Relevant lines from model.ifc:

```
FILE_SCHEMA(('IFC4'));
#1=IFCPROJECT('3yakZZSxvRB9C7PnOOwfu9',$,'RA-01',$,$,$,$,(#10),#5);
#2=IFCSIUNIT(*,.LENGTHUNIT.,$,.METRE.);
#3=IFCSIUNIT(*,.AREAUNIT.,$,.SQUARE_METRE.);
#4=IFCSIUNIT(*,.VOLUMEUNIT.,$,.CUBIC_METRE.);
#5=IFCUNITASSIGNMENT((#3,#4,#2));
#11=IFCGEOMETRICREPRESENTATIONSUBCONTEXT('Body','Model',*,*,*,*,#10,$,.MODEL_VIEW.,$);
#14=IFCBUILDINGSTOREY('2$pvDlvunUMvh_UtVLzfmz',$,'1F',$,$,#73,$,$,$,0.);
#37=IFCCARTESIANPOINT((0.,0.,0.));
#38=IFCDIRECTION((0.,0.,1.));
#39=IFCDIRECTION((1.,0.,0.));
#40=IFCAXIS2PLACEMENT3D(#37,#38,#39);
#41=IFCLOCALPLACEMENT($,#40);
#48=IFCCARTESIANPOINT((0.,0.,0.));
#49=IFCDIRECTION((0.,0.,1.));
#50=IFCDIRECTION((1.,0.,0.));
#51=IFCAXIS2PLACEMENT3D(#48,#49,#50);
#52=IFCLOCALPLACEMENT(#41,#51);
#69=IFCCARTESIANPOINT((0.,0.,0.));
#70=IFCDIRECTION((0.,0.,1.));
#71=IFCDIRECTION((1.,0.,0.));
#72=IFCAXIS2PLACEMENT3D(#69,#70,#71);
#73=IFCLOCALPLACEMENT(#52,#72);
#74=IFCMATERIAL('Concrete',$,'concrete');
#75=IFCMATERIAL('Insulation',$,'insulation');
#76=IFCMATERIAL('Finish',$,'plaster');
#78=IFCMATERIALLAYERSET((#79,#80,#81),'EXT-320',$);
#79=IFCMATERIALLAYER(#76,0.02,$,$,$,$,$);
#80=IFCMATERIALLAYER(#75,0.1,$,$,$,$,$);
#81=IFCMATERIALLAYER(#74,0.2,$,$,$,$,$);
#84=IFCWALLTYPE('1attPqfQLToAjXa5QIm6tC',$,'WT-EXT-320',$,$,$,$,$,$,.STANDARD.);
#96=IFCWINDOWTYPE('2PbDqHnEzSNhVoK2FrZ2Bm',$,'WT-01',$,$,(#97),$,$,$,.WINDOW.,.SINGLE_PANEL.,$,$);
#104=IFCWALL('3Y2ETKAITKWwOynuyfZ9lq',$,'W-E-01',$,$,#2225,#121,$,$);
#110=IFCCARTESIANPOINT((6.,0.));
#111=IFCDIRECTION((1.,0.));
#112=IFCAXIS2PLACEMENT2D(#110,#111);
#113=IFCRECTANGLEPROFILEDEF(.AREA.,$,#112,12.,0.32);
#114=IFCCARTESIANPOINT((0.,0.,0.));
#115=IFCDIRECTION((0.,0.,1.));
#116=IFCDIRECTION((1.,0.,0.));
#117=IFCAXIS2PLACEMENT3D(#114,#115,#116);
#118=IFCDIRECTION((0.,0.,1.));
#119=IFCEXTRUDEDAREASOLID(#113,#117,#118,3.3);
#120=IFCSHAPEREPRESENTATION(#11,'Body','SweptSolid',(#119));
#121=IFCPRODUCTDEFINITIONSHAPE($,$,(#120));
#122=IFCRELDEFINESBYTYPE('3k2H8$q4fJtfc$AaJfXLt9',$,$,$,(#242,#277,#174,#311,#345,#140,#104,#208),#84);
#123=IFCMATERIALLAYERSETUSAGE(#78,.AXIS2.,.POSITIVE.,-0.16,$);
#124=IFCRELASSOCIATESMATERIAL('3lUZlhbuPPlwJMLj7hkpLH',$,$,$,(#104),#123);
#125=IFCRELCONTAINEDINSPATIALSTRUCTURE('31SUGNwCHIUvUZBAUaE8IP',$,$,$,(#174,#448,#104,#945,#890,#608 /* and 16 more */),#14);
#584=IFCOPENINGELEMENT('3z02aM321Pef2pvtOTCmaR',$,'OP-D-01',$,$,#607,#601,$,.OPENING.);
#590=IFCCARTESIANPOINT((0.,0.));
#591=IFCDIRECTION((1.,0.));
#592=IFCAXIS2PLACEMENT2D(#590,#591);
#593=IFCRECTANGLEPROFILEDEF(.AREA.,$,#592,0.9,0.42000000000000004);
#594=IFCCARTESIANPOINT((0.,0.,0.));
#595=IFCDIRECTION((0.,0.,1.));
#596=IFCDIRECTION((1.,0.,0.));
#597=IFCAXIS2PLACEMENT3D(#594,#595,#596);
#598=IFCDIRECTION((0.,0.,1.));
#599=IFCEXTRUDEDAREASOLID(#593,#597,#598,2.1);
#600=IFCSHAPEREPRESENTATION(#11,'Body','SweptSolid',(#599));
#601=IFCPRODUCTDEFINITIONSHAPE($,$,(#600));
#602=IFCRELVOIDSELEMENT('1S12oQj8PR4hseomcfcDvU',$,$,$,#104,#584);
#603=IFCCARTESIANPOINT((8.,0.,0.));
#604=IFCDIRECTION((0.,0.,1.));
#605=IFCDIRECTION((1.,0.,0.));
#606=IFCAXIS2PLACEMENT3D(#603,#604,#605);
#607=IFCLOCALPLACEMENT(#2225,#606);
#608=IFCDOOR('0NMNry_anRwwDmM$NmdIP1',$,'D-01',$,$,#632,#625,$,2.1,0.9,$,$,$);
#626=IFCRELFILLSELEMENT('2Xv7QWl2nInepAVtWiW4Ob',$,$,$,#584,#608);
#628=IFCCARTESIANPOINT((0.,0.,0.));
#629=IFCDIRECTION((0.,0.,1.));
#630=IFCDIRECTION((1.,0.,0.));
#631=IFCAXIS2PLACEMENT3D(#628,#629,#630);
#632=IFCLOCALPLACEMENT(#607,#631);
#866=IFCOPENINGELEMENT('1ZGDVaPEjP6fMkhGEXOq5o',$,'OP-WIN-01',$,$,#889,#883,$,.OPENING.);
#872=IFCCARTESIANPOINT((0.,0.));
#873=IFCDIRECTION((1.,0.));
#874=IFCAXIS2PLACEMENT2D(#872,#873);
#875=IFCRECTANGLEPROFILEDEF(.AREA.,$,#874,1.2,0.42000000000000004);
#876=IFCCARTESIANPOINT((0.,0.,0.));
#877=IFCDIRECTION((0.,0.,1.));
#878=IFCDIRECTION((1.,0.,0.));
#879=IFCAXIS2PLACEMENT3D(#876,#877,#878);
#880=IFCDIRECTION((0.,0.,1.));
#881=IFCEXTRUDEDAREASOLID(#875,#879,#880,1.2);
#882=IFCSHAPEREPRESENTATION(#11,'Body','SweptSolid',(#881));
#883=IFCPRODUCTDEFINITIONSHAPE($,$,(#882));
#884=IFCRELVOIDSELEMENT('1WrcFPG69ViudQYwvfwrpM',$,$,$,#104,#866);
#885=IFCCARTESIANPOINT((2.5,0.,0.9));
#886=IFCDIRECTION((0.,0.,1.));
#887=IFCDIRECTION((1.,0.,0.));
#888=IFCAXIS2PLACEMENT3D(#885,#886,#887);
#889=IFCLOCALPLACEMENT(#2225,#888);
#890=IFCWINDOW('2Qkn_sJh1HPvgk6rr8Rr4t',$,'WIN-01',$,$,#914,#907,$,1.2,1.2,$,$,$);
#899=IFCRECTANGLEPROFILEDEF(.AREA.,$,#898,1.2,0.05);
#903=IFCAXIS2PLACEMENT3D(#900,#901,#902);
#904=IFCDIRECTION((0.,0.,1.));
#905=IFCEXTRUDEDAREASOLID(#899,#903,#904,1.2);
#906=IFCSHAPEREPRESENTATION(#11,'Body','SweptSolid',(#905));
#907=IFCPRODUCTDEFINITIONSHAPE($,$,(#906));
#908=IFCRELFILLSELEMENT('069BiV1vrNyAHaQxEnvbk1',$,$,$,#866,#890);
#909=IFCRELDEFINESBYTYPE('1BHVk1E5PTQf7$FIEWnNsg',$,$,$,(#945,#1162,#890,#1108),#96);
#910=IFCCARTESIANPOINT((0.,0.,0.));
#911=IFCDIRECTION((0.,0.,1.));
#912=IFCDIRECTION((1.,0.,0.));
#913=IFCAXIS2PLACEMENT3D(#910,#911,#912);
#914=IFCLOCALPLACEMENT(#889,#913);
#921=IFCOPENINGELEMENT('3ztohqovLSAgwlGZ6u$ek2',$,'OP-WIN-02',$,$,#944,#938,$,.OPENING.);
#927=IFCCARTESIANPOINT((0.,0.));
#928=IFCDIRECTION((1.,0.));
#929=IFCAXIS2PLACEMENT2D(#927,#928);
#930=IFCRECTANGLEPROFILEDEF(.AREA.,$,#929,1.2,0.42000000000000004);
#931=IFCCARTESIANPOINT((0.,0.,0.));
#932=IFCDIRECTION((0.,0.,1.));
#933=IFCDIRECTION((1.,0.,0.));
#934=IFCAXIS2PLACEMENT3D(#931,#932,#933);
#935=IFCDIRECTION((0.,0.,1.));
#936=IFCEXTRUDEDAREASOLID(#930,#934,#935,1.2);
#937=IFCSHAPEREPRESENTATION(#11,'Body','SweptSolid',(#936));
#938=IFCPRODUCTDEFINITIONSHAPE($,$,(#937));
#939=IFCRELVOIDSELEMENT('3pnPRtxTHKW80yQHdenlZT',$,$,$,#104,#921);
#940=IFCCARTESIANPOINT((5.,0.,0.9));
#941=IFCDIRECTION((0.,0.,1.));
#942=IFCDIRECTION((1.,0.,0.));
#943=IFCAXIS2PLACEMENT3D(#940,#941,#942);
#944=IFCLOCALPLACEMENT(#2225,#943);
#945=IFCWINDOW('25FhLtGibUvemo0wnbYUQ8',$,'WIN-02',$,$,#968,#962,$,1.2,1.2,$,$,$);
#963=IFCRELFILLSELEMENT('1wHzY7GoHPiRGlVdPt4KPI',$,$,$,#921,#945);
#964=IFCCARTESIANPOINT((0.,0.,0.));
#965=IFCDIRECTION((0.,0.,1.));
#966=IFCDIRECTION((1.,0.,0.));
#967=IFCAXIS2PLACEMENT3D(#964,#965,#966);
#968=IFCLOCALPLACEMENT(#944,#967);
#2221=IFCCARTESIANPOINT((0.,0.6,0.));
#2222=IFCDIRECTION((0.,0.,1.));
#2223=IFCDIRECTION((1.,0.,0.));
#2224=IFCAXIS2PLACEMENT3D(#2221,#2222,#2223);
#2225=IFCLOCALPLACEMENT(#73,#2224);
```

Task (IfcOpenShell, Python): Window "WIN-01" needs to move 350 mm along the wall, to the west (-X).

```python
import ifcopenshell
import ifcopenshell.api.geometry
import ifcopenshell.util.placement
import ifcopenshell.util.unit

model = ifcopenshell.open("model.ifc")
unit_scale = ifcopenshell.util.unit.calculate_unit_scale(model)

window = model.by_guid("2Qkn_sJh1HPvgk6rr8Rr4t")
opening = window.FillsVoids[0].RelatingOpeningElement
wall = opening.VoidsElements[0].RelatingBuildingElement

wall_matrix = ifcopenshell.util.placement.get_local_placement(wall.ObjectPlacement)
shift = wall_matrix[:3, 0] * -0.35 / unit_scale
before = ifcopenshell.util.placement.get_local_placement(window.ObjectPlacement)[:3, 3].copy()

# The window is placed relative to its opening, so it follows when the opening moves.
matrix = ifcopenshell.util.placement.get_local_placement(opening.ObjectPlacement)
matrix[:3, 3] += shift
ifcopenshell.api.geometry.edit_object_placement(
    model, product=opening, matrix=matrix, is_si=False, should_transform_children=True
)

after = ifcopenshell.util.placement.get_local_placement(window.ObjectPlacement)[:3, 3]
print("window moved by", (after - before).round(3) + 0.0)

model.write("model-out.ifc")
```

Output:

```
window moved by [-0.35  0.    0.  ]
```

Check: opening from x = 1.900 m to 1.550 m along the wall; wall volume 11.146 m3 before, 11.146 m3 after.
